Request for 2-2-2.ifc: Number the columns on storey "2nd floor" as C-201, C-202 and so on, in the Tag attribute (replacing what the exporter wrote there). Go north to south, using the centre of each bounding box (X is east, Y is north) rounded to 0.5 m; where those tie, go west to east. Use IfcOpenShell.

First a look at what the model holds.

```python
import ifcopenshell
import ifcopenshell.util.element
import ifcopenshell.util.placement

model = ifcopenshell.open("2-2-2.ifc")
print(model.schema)
storey = next(s for s in model.by_type("IfcBuildingStorey") if s.Name == "2nd floor")
columns = [e for e in ifcopenshell.util.element.get_decomposition(storey) if e.is_a("IfcColumn")]
for e in sorted(columns, key=lambda e: e.id()):
    origin = ifcopenshell.util.placement.get_local_placement(e.ObjectPlacement)[:3, 3]
    print(e.id(), e.Tag, e.Name, origin.round(2) + 0.0, sep=" | ")
```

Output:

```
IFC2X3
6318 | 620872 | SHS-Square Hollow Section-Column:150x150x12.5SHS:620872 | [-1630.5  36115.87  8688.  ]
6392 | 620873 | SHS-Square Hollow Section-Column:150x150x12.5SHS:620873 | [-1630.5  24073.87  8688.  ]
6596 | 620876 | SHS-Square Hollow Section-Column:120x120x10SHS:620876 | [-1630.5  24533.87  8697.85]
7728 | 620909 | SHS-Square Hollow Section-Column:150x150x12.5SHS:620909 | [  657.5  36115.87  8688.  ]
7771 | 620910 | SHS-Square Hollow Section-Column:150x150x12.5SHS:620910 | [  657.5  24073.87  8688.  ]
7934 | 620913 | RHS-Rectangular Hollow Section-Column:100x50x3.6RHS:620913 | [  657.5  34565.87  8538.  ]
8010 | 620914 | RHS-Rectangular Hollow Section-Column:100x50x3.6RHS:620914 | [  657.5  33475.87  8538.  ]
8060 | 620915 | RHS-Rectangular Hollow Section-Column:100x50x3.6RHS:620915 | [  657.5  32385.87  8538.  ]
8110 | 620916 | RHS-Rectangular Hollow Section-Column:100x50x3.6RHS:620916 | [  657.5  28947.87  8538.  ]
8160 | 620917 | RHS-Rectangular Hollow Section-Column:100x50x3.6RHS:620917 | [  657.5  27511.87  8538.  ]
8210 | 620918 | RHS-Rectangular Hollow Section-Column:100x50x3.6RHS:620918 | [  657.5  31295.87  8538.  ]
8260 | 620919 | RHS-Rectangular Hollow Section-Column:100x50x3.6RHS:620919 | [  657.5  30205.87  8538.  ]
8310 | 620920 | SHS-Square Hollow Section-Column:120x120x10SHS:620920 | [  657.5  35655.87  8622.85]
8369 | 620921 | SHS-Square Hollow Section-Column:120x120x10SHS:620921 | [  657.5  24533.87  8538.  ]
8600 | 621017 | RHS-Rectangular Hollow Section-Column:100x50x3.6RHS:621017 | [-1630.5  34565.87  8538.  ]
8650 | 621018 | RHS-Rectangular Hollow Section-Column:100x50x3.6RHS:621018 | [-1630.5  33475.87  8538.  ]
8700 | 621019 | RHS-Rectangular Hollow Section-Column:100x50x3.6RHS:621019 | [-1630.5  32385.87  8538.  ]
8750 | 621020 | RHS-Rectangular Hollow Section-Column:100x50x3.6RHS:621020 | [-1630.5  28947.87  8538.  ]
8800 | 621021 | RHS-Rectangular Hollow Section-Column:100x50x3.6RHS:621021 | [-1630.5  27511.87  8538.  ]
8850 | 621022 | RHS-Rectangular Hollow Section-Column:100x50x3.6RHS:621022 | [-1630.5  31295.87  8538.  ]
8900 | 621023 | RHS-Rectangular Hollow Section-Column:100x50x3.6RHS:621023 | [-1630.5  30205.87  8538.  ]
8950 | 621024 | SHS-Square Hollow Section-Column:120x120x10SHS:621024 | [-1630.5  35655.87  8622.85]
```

```python
import ifcopenshell
import ifcopenshell.geom
import ifcopenshell.util.element
import ifcopenshell.util.shape

model = ifcopenshell.open("2-2-2.ifc")
settings = ifcopenshell.geom.settings()
settings.set("use-world-coords", True)


def centre(element):
    shape = ifcopenshell.geom.create_shape(settings, element)
    return ifcopenshell.util.shape.get_bbox_centroid(shape.geometry)


storey = next(s for s in model.by_type("IfcBuildingStorey") if s.Name == "2nd floor")
columns = [e for e in ifcopenshell.util.element.get_decomposition(storey) if e.is_a("IfcColumn")]

# Insertion points can sit at a corner or the storey origin, so sort by the geometry (in metres).
centres = {e: centre(e) for e in columns}
columns.sort(key=lambda e: (-round(centres[e][1] / 0.5), centres[e][0]))

for i, e in enumerate(columns, start=1):
    number = f"C-2{i:02d}"
    e.Tag = number
    print(e.id(), number)

model.write("2-2-2_rev.ifc")
```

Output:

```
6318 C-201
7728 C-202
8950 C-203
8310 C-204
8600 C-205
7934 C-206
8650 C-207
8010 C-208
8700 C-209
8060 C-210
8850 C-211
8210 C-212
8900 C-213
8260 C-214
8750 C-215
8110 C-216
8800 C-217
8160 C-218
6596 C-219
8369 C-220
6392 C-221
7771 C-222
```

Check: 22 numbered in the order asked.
